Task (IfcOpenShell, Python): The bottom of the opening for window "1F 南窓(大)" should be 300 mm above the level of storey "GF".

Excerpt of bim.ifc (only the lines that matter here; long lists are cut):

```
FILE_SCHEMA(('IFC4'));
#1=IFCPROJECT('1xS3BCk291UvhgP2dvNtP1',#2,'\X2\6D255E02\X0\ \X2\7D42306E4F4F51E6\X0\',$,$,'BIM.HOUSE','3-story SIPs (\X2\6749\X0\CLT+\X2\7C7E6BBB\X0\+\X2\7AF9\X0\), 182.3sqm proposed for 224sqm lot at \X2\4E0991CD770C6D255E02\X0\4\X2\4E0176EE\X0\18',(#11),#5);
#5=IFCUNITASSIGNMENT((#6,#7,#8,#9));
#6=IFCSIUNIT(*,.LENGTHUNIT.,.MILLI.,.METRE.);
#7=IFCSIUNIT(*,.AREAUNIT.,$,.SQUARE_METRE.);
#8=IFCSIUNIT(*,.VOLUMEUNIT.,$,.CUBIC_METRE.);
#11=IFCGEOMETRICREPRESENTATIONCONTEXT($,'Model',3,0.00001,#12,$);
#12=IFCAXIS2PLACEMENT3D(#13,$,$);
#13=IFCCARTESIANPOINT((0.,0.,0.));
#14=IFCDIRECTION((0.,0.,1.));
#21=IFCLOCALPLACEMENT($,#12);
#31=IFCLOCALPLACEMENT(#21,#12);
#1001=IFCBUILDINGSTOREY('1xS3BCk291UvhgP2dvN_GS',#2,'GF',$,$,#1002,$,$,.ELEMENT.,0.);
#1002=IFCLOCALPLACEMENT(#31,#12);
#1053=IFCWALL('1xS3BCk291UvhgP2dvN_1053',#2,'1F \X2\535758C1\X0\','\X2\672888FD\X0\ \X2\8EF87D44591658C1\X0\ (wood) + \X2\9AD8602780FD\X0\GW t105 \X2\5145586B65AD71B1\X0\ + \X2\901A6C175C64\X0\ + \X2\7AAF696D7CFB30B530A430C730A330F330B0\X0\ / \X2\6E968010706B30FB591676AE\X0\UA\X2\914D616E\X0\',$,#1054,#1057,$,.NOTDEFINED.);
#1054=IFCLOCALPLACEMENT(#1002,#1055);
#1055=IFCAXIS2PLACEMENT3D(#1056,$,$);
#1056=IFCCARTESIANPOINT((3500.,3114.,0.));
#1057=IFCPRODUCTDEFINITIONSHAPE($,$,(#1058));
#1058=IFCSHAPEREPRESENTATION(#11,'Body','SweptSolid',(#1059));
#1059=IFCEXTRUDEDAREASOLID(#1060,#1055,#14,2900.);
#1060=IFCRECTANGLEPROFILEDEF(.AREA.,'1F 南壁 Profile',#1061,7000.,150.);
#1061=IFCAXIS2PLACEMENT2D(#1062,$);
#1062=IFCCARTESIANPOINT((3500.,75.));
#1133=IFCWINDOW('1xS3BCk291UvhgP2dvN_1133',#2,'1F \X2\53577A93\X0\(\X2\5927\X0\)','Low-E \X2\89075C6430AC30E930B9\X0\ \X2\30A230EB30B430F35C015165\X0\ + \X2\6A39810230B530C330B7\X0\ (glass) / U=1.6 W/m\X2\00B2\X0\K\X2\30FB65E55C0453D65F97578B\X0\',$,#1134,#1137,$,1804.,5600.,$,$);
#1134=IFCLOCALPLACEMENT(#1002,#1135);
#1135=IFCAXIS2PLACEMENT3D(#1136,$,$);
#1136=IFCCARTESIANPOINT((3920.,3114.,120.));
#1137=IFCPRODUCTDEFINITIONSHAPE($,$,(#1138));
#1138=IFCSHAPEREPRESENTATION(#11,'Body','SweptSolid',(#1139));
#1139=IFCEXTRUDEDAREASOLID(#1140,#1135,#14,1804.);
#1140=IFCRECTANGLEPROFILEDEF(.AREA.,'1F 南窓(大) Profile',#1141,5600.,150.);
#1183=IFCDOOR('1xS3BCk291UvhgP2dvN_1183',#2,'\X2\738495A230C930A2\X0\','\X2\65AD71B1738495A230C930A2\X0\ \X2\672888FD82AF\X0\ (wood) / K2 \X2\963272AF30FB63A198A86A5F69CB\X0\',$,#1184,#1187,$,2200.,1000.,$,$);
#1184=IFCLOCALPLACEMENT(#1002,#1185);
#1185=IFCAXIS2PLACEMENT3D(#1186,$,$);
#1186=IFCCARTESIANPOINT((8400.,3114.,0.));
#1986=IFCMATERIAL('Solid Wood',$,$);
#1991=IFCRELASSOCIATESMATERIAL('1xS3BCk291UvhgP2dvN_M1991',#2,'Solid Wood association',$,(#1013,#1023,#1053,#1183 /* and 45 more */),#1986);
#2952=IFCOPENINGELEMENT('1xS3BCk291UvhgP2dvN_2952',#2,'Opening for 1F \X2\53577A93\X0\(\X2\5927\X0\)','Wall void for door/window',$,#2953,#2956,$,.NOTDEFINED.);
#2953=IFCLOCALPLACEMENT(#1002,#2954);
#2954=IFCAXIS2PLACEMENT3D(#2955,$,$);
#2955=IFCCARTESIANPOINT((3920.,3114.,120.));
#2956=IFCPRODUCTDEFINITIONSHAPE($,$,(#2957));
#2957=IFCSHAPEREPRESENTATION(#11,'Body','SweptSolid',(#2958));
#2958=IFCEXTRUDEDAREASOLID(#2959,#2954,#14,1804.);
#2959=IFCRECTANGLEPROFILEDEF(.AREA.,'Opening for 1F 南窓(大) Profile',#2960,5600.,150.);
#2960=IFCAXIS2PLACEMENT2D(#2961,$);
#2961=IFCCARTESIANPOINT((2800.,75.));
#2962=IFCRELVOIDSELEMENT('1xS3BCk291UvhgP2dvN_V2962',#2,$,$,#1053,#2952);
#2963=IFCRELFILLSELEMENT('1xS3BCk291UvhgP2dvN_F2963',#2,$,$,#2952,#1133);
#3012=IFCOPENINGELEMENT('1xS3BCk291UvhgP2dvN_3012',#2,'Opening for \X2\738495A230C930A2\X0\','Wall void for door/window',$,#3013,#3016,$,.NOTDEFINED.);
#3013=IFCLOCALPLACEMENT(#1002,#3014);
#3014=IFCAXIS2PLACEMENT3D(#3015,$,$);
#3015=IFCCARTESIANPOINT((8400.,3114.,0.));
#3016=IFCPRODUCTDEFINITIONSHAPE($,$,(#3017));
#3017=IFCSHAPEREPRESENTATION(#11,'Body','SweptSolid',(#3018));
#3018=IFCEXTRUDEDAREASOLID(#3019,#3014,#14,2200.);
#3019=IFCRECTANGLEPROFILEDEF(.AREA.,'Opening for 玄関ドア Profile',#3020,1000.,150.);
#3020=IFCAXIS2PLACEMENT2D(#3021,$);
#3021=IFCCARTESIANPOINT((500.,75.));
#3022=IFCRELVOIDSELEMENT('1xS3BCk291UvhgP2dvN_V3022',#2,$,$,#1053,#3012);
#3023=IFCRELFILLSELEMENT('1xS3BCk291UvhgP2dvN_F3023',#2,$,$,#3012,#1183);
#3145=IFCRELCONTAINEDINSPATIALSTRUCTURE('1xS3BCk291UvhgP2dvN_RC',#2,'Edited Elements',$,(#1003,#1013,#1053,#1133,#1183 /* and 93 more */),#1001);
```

```python
import numpy as np
import ifcopenshell
import ifcopenshell.api.geometry
import ifcopenshell.geom
import ifcopenshell.util.element
import ifcopenshell.util.placement
import ifcopenshell.util.shape
import ifcopenshell.util.unit

model = ifcopenshell.open("bim.ifc")
unit_scale = ifcopenshell.util.unit.calculate_unit_scale(model)

window = model.by_guid("1xS3BCk291UvhgP2dvN_1133")
opening = window.FillsVoids[0].RelatingOpeningElement
storey = ifcopenshell.util.element.get_container(window, ifc_class="IfcBuildingStorey")
level = ifcopenshell.util.placement.get_local_placement(storey.ObjectPlacement)[2, 3]

# The opening's origin need not be at the sill, so measure its lowest point.
shape = ifcopenshell.geom.create_shape(ifcopenshell.geom.settings(), opening)
bottom = ifcopenshell.util.shape.get_shape_bottom_elevation(shape, shape.geometry) / unit_scale
dz = level + 0.3 / unit_scale - bottom

shift = np.array([0.0, 0.0, dz])
# The window is not placed relative to its opening, so move both.
for product in (opening, window):
    matrix = ifcopenshell.util.placement.get_local_placement(product.ObjectPlacement)
    matrix[:3, 3] += shift
    ifcopenshell.api.geometry.edit_object_placement(model, product=product, matrix=matrix, is_si=False)

print(f"moved by {dz * unit_scale:+.3f} m")

model.write("bim_rev.ifc")
```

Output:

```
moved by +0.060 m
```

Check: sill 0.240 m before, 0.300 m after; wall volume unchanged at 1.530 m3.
